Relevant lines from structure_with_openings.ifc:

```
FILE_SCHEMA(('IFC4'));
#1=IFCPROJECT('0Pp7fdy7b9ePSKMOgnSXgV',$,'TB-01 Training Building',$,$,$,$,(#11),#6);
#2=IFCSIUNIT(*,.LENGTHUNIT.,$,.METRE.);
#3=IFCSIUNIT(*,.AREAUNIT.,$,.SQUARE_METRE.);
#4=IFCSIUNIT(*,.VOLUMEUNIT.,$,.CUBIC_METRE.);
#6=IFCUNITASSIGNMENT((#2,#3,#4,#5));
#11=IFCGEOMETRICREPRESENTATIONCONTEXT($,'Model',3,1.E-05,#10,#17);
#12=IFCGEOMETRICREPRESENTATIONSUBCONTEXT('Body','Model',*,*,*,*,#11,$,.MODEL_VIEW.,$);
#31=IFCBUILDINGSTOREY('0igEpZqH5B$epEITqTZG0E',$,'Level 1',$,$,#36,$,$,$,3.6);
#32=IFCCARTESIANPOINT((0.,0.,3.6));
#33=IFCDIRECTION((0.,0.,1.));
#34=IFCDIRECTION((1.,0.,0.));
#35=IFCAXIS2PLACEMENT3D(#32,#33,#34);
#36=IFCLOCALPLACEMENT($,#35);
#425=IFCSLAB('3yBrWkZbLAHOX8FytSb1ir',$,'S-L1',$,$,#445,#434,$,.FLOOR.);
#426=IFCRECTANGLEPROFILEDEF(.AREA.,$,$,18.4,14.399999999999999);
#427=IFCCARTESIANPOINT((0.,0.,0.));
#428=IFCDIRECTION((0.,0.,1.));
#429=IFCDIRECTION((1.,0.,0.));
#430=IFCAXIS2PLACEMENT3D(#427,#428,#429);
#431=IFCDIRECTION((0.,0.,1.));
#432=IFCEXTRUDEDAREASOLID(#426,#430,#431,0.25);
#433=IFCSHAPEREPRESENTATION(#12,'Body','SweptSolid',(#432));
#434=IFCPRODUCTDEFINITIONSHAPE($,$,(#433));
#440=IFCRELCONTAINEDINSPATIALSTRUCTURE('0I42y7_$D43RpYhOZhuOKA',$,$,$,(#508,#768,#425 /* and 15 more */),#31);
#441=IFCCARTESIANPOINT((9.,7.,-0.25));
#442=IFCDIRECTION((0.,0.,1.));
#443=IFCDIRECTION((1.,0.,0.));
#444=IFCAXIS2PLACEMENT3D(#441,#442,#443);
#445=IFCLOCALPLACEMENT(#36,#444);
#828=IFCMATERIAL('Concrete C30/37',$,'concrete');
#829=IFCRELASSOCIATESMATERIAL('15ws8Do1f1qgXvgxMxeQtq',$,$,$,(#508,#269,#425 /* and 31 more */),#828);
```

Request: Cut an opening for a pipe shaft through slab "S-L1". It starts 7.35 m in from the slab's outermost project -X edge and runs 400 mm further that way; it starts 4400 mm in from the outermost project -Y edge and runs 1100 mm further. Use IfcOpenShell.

```python
import numpy as np
import ifcopenshell
import ifcopenshell.api.feature
import ifcopenshell.api.geometry
import ifcopenshell.api.root
import ifcopenshell.geom
import ifcopenshell.util.placement
import ifcopenshell.util.representation
import ifcopenshell.util.shape
import ifcopenshell.util.unit

model = ifcopenshell.open("structure_with_openings.ifc")
unit_scale = ifcopenshell.util.unit.calculate_unit_scale(model)
settings = ifcopenshell.geom.settings()


def volume(element):
    """Net volume in cubic metres, openings subtracted."""
    shape = ifcopenshell.geom.create_shape(settings, element)
    return ifcopenshell.util.shape.get_volume(shape.geometry)


slab = model.by_id(425)
before = volume(slab)

# Extent in the slab's own axes, in metres. The edges named are its -X and -Y sides.
slab_shape = ifcopenshell.geom.create_shape(settings, slab)
vertices = ifcopenshell.util.shape.get_vertices(slab_shape.geometry)
x_min, y_min, bottom = vertices.min(axis=0)
top = vertices[:, 2].max()

opening = ifcopenshell.api.root.create_entity(model, ifc_class="IfcOpeningElement", name="Pipe shaft opening", predefined_type="OPENING")
context = ifcopenshell.util.representation.get_context(model, "Model", "Body", "MODEL_VIEW")
width, depth = 0.4, 1.1
outline = [(0.0, 0.0), (width, 0.0), (width, depth), (0.0, depth), (0.0, 0.0)]
# Overshoot both faces by 50 mm so the cut is clean.
shape = ifcopenshell.api.geometry.add_slab_representation(
    model, context=context, depth=top - bottom + 0.1, polyline=outline
)
ifcopenshell.api.geometry.assign_representation(model, product=opening, representation=shape)

matrix = ifcopenshell.util.placement.get_local_placement(slab.ObjectPlacement)
matrix[:, 3] = matrix @ np.append(np.array([x_min + 7.35, y_min + 4.4, bottom - 0.05]) / unit_scale, 1.0)
ifcopenshell.api.geometry.edit_object_placement(model, product=opening, matrix=matrix, is_si=False)
ifcopenshell.api.feature.add_feature(model, feature=opening, element=slab)

after = volume(slab)

print(f"slab volume {before:.3f} -> {after:.3f} m3")

model.write("structure_with_openings_rev.ifc")
```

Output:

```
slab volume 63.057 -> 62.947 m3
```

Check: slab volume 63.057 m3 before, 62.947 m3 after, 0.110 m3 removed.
